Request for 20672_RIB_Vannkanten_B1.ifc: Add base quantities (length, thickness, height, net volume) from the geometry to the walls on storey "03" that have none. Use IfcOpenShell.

First a look at what the model holds.

```python
import ifcopenshell
import ifcopenshell.util.element
import ifcopenshell.util.unit

model = ifcopenshell.open("20672_RIB_Vannkanten_B1.ifc")
print(model.schema)
for unit_type in ("LENGTHUNIT", "AREAUNIT", "VOLUMEUNIT"):
    print(unit_type, ifcopenshell.util.unit.calculate_unit_scale(model, unit_type))
storey = next(s for s in model.by_type("IfcBuildingStorey") if s.Name == "03")
walls = [e for e in ifcopenshell.util.element.get_decomposition(storey) if e.is_a("IfcWall")]
for e in sorted(walls, key=lambda e: e.id()):
    print(e.id(), e.is_a(), e.Name, list(ifcopenshell.util.element.get_psets(e, qtos_only=True)), sep=" | ")
```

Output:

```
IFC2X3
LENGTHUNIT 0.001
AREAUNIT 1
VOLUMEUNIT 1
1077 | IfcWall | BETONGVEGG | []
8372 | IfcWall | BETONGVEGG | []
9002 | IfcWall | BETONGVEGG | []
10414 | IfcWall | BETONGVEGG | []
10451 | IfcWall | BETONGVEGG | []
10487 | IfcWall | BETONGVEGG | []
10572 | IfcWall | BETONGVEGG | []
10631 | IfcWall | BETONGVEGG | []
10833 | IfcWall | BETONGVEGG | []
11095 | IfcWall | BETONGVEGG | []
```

```python
import ifcopenshell
import ifcopenshell.api.pset
import ifcopenshell.geom
import ifcopenshell.util.element
import ifcopenshell.util.shape
import ifcopenshell.util.unit

model = ifcopenshell.open("20672_RIB_Vannkanten_B1.ifc")
unit_scale = ifcopenshell.util.unit.calculate_unit_scale(model)
volume_scale = ifcopenshell.util.unit.calculate_unit_scale(model, "VOLUMEUNIT")
settings = ifcopenshell.geom.settings()

storey = next(s for s in model.by_type("IfcBuildingStorey") if s.Name == "03")
walls = [e for e in ifcopenshell.util.element.get_decomposition(storey) if e.is_a("IfcWall")]

for e in sorted(walls, key=lambda e: e.id()):
    if ifcopenshell.util.element.get_psets(e, qtos_only=True, should_inherit=False):
        continue
    # Geometry comes back in metres, in the element's own axes.
    shape = ifcopenshell.geom.create_shape(settings, e)
    values = {
        "Length": ifcopenshell.util.shape.get_x(shape.geometry) / unit_scale,
        "Width": ifcopenshell.util.shape.get_y(shape.geometry) / unit_scale,
        "Height": ifcopenshell.util.shape.get_z(shape.geometry) / unit_scale,
        "NetVolume": ifcopenshell.util.shape.get_volume(shape.geometry) / volume_scale,
    }
    qto = ifcopenshell.api.pset.add_qto(model, product=e, name="BaseQuantities")
    ifcopenshell.api.pset.edit_qto(model, qto=qto, properties=values)
    print(e.id(), {k: round(v, 3) for k, v in values.items()})

model.write("20672_RIB_Vannkanten_B1_edited.ifc")
```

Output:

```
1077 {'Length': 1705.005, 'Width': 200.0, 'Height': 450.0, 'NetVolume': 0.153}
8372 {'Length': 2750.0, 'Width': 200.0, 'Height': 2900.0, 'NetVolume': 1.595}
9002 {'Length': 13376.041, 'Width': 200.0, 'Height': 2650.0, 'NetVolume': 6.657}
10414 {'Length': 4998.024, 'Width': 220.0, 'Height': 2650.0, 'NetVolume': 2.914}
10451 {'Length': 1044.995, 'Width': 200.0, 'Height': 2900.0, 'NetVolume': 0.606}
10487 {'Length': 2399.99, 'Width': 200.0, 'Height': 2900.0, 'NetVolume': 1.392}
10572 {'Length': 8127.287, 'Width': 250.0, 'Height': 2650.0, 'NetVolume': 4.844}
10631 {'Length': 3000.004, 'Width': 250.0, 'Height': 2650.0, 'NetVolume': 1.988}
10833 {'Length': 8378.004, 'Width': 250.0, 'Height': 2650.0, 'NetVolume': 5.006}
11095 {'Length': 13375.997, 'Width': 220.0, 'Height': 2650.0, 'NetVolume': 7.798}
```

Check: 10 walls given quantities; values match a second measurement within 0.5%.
